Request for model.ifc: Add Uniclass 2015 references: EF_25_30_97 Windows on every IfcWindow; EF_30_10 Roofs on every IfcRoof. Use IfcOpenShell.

First a look at what the model holds.

```python
import ifcopenshell

model = ifcopenshell.open("model.ifc")
print(model.schema)
print("classifications:", [c.Name for c in model.by_type("IfcClassification")])
for ifc_class in ("IfcDoor", "IfcRoof", "IfcStair", "IfcWall", "IfcWindow"):
    print(ifc_class, len(model.by_type(ifc_class)))
```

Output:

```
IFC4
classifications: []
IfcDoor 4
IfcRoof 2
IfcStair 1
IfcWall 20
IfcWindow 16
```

```python
import ifcopenshell
import ifcopenshell.api.classification

model = ifcopenshell.open("model.ifc")

system = ifcopenshell.api.classification.add_classification(model, classification="Uniclass 2015")

codes = {
    "IfcWindow": ("EF_25_30_97", "Windows"),
    "IfcRoof": ("EF_30_10", "Roofs"),
}
for ifc_class, (code, name) in codes.items():
    products = model.by_type(ifc_class)
    ifcopenshell.api.classification.add_reference(
        model, products=products, classification=system, identification=code, name=name
    )
    print(code, len(products))

model.write("model_updated.ifc")
```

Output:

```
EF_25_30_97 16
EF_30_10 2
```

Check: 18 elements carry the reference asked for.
